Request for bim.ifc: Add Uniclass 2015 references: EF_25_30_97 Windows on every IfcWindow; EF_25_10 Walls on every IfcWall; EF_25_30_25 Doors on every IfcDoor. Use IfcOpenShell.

First a look at what the model holds.

```python
import ifcopenshell

model = ifcopenshell.open("bim.ifc")
print(model.schema)
print("classifications:", [c.Name for c in model.by_type("IfcClassification")])
for ifc_class in ("IfcDoor", "IfcRoof", "IfcStair", "IfcWall", "IfcWindow"):
    print(ifc_class, len(model.by_type(ifc_class)))
```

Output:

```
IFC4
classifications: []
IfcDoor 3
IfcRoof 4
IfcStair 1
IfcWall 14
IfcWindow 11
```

```python
import ifcopenshell
import ifcopenshell.api.classification

model = ifcopenshell.open("bim.ifc")

system = ifcopenshell.api.classification.add_classification(model, classification="Uniclass 2015")

codes = {
    "IfcWindow": ("EF_25_30_97", "Windows"),
    "IfcWall": ("EF_25_10", "Walls"),
    "IfcDoor": ("EF_25_30_25", "Doors"),
}
for ifc_class, (code, name) in codes.items():
    products = model.by_type(ifc_class)
    ifcopenshell.api.classification.add_reference(
        model, products=products, classification=system, identification=code, name=name
    )
    print(code, len(products))

model.write("bim_edited.ifc")
```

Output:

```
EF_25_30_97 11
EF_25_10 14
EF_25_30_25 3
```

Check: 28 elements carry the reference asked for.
